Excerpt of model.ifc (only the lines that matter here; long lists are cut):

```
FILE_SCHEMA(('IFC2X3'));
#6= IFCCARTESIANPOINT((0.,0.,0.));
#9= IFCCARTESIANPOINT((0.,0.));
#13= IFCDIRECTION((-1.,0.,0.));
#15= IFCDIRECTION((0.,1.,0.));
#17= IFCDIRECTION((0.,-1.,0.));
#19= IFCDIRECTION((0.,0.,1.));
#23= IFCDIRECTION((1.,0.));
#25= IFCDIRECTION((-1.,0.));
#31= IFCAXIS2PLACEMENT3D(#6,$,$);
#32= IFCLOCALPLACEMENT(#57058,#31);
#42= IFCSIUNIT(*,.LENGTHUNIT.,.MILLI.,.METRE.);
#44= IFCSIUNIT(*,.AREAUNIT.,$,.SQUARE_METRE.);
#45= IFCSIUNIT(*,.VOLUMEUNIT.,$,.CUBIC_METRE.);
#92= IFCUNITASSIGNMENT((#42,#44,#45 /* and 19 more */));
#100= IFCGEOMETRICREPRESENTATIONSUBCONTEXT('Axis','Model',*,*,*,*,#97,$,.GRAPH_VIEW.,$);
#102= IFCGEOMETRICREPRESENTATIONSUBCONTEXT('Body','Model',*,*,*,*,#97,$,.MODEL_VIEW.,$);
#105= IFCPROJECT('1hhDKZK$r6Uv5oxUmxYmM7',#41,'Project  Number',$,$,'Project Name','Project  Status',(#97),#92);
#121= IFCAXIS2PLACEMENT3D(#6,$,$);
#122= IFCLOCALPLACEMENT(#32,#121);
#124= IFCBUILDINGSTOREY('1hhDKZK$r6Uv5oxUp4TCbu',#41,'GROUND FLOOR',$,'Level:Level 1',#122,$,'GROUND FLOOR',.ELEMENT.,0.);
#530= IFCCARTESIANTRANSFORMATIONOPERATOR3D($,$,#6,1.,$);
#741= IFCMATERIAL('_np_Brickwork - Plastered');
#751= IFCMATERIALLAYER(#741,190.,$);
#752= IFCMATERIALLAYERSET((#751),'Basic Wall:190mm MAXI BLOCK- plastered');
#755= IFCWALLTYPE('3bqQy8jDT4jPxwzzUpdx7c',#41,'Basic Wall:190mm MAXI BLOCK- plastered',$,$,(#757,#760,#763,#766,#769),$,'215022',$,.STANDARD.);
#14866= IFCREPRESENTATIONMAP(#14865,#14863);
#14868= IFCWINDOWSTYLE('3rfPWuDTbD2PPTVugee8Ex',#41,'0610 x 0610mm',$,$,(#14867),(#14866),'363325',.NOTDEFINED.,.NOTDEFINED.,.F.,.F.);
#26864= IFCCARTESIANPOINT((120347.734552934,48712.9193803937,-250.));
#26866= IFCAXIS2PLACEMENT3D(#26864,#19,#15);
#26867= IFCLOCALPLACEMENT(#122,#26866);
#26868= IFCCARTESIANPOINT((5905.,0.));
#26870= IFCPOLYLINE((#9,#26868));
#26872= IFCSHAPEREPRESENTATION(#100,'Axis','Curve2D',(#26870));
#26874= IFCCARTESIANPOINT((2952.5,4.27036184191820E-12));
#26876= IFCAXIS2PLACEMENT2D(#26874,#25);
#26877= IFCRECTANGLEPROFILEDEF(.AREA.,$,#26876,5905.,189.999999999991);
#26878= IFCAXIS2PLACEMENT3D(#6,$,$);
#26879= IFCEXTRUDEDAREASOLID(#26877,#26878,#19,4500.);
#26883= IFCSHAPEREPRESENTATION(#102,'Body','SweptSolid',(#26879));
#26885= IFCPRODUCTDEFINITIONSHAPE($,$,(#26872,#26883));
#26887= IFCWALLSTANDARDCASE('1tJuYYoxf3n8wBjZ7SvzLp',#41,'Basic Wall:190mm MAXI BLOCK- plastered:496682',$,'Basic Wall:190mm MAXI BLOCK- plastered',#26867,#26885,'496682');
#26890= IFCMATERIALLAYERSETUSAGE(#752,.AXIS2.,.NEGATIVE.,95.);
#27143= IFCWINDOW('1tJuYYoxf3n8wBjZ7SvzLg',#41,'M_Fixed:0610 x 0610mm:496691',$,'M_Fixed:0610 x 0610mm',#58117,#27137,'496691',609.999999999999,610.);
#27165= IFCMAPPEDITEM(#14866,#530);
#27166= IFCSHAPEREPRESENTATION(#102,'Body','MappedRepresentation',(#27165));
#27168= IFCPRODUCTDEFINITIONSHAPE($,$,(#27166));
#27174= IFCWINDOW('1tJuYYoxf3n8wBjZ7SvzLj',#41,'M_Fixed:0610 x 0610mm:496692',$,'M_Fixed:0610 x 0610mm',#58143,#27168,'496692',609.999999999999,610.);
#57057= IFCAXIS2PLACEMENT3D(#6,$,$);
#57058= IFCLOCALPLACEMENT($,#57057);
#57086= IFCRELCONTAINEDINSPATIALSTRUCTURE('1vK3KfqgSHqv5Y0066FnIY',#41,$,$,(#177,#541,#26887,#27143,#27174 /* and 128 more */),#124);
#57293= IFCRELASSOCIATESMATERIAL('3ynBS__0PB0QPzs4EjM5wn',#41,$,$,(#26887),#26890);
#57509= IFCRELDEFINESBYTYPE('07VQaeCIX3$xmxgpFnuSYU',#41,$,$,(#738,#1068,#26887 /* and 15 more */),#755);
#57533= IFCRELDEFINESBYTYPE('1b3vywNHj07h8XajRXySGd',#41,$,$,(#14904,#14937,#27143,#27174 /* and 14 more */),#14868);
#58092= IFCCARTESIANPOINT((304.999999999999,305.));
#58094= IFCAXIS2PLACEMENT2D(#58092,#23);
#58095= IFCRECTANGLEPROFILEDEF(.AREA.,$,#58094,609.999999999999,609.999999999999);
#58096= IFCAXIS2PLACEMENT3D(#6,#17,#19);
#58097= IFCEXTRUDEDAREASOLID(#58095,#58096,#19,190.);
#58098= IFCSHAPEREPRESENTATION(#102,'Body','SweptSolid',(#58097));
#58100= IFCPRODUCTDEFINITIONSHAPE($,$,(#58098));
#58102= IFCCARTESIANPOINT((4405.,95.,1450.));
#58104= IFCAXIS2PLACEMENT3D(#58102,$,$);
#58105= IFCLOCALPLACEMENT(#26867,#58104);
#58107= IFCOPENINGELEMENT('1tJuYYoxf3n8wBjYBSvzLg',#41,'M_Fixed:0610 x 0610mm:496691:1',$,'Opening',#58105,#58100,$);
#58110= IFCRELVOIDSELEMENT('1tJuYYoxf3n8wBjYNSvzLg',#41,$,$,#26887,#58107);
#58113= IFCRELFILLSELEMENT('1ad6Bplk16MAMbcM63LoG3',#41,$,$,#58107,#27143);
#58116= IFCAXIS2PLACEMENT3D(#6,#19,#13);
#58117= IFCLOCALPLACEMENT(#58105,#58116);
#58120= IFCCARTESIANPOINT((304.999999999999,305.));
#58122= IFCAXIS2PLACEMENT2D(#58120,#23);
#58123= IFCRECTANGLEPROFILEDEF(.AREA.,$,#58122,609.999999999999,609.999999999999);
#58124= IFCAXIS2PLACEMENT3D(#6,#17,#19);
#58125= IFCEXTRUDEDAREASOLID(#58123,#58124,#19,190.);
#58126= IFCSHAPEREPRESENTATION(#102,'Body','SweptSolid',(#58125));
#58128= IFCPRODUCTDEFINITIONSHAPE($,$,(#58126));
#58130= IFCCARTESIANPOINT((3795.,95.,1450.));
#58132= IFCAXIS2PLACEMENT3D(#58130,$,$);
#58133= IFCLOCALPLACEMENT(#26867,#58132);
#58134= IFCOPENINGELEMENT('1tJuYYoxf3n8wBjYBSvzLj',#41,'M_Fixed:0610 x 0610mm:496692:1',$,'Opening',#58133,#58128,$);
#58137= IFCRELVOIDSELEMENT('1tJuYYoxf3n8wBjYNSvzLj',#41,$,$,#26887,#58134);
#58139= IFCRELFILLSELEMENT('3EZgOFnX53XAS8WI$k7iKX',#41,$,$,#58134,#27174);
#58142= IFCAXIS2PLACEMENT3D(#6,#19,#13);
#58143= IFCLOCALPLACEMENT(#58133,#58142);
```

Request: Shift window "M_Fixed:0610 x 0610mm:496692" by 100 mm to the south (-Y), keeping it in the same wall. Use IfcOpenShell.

```python
import ifcopenshell
import ifcopenshell.api.geometry
import ifcopenshell.util.placement
import ifcopenshell.util.unit

model = ifcopenshell.open("model.ifc")
unit_scale = ifcopenshell.util.unit.calculate_unit_scale(model)

window = model.by_guid("1tJuYYoxf3n8wBjZ7SvzLj")
opening = window.FillsVoids[0].RelatingOpeningElement
wall = opening.VoidsElements[0].RelatingBuildingElement

wall_matrix = ifcopenshell.util.placement.get_local_placement(wall.ObjectPlacement)
shift = wall_matrix[:3, 0] * -0.1 / unit_scale
before = ifcopenshell.util.placement.get_local_placement(window.ObjectPlacement)[:3, 3].copy()

# The window is placed relative to its opening, so it follows when the opening moves.
matrix = ifcopenshell.util.placement.get_local_placement(opening.ObjectPlacement)
matrix[:3, 3] += shift
ifcopenshell.api.geometry.edit_object_placement(
    model, product=opening, matrix=matrix, is_si=False, should_transform_children=True
)

after = ifcopenshell.util.placement.get_local_placement(window.ObjectPlacement)[:3, 3]
print("window moved by", (after - before).round(3) + 0.0)

model.write("model_updated.ifc")
```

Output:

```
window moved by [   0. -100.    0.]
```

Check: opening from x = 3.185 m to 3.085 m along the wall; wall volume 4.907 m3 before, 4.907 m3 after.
